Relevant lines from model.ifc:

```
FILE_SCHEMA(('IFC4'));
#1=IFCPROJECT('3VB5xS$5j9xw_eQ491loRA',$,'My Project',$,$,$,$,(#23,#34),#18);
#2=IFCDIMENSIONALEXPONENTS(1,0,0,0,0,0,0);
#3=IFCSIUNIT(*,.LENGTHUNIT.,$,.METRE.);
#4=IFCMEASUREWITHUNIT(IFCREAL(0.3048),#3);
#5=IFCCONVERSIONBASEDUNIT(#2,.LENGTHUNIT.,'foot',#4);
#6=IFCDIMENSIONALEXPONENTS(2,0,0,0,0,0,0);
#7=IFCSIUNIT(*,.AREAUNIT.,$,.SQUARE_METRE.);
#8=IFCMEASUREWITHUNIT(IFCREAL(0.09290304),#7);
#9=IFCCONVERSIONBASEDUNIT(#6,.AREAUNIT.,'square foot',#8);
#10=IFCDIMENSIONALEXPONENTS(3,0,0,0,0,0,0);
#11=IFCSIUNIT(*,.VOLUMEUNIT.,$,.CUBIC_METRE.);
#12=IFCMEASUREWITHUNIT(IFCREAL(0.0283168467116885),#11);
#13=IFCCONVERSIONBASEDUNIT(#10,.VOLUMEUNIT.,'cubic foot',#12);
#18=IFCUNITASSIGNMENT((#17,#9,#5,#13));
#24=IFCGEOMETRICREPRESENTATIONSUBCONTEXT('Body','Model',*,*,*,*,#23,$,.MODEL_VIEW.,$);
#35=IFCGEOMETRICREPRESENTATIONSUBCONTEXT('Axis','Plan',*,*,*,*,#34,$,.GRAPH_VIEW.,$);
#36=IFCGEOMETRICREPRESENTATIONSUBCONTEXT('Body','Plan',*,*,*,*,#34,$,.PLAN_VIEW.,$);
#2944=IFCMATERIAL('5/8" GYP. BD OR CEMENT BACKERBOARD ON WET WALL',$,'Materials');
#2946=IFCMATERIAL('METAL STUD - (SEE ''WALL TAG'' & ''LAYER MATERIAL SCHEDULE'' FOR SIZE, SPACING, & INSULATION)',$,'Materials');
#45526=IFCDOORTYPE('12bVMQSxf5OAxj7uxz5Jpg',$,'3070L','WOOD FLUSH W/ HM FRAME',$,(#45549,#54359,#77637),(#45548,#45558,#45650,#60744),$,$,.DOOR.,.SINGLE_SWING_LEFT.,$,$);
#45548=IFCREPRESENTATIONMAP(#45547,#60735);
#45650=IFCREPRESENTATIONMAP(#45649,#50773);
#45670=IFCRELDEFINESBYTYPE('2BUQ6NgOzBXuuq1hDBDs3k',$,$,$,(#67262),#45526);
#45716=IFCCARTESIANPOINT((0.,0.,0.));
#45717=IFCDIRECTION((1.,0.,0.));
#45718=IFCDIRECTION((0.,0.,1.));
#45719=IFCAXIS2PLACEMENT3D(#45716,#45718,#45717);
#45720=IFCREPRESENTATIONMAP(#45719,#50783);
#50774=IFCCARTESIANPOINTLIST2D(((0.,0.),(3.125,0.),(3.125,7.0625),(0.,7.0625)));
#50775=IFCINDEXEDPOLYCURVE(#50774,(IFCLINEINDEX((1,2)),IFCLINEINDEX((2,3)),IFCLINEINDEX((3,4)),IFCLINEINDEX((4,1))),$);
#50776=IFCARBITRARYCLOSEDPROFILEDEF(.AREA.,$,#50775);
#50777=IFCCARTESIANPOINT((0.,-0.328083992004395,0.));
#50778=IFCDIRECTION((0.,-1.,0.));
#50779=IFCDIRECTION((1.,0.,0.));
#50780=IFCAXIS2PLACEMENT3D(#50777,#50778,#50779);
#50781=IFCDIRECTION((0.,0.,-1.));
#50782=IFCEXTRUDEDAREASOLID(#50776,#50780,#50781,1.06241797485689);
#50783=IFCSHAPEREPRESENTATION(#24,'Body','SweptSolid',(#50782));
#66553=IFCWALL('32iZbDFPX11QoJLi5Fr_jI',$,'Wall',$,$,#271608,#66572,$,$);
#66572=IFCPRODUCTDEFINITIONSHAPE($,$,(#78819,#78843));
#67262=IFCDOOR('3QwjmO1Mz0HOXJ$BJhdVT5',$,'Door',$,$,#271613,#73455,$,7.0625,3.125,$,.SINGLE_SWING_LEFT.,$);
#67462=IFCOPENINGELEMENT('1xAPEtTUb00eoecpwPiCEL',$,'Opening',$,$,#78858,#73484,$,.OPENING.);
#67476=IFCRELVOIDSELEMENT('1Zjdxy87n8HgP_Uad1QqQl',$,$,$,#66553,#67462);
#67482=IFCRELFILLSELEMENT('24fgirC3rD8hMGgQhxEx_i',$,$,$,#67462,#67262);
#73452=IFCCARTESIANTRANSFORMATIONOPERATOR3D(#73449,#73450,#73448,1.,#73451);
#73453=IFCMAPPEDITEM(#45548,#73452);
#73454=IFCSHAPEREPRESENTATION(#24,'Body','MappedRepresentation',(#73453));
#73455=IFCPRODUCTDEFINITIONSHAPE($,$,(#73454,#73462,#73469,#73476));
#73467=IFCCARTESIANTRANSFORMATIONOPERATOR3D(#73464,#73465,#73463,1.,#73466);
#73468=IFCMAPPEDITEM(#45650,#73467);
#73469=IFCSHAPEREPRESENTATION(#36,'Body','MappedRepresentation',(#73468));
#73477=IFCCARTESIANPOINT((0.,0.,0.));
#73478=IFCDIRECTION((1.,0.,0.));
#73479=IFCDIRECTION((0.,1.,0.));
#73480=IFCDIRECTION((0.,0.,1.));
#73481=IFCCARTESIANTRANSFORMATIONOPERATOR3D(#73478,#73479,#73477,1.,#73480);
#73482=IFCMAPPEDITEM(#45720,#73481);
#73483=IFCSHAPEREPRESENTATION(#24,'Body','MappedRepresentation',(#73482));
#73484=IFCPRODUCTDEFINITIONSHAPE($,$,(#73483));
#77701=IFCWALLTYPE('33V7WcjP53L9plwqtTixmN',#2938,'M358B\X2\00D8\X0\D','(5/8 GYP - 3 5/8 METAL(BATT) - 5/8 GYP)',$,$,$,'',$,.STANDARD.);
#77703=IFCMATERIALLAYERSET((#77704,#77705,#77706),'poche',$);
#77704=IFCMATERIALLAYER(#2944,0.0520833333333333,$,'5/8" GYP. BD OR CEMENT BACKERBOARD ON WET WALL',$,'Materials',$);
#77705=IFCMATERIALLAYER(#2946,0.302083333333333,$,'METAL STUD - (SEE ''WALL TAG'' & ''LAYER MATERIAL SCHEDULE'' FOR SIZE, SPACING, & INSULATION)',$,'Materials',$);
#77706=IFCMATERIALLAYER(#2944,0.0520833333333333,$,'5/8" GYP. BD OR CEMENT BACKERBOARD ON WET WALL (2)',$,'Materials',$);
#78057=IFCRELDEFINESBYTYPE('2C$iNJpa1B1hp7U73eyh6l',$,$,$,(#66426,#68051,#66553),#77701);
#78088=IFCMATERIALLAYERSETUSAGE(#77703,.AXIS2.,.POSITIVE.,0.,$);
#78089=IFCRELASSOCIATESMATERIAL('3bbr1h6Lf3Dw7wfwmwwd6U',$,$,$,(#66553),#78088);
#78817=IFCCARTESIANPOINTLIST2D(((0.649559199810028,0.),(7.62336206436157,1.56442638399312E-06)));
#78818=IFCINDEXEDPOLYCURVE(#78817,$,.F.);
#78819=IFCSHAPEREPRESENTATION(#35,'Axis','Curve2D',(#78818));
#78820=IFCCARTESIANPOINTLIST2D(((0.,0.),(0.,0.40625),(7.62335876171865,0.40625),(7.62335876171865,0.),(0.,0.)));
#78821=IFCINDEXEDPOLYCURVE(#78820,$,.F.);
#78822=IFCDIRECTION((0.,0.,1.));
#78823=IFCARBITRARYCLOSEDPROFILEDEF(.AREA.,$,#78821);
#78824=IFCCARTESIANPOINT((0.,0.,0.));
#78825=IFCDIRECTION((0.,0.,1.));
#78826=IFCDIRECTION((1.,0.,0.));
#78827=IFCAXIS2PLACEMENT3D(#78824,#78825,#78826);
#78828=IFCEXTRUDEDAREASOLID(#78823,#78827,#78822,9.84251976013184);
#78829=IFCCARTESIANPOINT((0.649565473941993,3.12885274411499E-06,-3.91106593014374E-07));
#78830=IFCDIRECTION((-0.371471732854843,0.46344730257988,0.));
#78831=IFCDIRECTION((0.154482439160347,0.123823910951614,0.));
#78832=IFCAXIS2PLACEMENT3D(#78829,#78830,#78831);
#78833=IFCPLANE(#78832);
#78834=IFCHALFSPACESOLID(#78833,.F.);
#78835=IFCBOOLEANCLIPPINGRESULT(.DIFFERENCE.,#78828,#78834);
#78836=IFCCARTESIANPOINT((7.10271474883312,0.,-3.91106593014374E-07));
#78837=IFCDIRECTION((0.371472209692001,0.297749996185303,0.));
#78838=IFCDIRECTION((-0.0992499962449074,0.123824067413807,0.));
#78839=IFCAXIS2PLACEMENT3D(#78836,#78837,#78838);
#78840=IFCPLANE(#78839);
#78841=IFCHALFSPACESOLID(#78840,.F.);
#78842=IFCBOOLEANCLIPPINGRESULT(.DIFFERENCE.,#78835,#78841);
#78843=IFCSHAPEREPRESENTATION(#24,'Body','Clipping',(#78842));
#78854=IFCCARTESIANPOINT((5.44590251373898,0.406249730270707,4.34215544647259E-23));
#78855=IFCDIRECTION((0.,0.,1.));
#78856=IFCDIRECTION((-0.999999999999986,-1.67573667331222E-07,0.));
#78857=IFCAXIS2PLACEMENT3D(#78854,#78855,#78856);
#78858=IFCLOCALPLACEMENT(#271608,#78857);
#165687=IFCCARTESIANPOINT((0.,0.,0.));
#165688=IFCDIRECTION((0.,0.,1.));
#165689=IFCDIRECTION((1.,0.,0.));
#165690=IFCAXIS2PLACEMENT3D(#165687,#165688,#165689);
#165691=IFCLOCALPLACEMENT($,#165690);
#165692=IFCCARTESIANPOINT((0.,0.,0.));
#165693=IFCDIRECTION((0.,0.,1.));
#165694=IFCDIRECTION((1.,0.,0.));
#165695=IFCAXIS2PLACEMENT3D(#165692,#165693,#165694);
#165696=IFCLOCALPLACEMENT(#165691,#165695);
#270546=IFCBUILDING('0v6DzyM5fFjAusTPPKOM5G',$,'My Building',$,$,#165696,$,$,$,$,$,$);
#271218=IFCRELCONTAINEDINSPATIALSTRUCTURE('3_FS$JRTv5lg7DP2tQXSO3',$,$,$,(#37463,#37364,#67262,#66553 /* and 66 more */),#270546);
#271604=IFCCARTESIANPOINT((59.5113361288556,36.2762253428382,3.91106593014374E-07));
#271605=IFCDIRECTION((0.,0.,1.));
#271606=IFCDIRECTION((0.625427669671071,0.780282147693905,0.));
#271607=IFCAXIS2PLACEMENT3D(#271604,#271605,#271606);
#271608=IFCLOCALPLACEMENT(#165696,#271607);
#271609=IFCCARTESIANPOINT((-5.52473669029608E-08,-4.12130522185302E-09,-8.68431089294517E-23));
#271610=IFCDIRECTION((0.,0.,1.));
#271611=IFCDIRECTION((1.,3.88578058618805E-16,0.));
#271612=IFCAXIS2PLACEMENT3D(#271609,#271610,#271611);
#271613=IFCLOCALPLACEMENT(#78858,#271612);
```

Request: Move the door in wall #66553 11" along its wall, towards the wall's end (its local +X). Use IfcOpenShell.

```python
import ifcopenshell
import ifcopenshell.api.geometry
import ifcopenshell.util.placement
import ifcopenshell.util.unit

model = ifcopenshell.open("model.ifc")
unit_scale = ifcopenshell.util.unit.calculate_unit_scale(model)

door = model.by_guid("3QwjmO1Mz0HOXJ$BJhdVT5")
opening = door.FillsVoids[0].RelatingOpeningElement
wall = opening.VoidsElements[0].RelatingBuildingElement

wall_matrix = ifcopenshell.util.placement.get_local_placement(wall.ObjectPlacement)
shift = wall_matrix[:3, 0] * 11 * 0.0254 / unit_scale
before = ifcopenshell.util.placement.get_local_placement(door.ObjectPlacement)[:3, 3].copy()

# The door is placed relative to its opening, so it follows when the opening moves.
matrix = ifcopenshell.util.placement.get_local_placement(opening.ObjectPlacement)
matrix[:3, 3] += shift
ifcopenshell.api.geometry.edit_object_placement(
    model, product=opening, matrix=matrix, is_si=False, should_transform_children=True
)

after = ifcopenshell.util.placement.get_local_placement(door.ObjectPlacement)[:3, 3]
print("door moved by", (after - before).round(3) + 0.0)

model.write("model-out.ifc")
```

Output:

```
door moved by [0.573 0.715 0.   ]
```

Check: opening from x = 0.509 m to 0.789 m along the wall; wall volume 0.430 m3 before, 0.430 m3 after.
